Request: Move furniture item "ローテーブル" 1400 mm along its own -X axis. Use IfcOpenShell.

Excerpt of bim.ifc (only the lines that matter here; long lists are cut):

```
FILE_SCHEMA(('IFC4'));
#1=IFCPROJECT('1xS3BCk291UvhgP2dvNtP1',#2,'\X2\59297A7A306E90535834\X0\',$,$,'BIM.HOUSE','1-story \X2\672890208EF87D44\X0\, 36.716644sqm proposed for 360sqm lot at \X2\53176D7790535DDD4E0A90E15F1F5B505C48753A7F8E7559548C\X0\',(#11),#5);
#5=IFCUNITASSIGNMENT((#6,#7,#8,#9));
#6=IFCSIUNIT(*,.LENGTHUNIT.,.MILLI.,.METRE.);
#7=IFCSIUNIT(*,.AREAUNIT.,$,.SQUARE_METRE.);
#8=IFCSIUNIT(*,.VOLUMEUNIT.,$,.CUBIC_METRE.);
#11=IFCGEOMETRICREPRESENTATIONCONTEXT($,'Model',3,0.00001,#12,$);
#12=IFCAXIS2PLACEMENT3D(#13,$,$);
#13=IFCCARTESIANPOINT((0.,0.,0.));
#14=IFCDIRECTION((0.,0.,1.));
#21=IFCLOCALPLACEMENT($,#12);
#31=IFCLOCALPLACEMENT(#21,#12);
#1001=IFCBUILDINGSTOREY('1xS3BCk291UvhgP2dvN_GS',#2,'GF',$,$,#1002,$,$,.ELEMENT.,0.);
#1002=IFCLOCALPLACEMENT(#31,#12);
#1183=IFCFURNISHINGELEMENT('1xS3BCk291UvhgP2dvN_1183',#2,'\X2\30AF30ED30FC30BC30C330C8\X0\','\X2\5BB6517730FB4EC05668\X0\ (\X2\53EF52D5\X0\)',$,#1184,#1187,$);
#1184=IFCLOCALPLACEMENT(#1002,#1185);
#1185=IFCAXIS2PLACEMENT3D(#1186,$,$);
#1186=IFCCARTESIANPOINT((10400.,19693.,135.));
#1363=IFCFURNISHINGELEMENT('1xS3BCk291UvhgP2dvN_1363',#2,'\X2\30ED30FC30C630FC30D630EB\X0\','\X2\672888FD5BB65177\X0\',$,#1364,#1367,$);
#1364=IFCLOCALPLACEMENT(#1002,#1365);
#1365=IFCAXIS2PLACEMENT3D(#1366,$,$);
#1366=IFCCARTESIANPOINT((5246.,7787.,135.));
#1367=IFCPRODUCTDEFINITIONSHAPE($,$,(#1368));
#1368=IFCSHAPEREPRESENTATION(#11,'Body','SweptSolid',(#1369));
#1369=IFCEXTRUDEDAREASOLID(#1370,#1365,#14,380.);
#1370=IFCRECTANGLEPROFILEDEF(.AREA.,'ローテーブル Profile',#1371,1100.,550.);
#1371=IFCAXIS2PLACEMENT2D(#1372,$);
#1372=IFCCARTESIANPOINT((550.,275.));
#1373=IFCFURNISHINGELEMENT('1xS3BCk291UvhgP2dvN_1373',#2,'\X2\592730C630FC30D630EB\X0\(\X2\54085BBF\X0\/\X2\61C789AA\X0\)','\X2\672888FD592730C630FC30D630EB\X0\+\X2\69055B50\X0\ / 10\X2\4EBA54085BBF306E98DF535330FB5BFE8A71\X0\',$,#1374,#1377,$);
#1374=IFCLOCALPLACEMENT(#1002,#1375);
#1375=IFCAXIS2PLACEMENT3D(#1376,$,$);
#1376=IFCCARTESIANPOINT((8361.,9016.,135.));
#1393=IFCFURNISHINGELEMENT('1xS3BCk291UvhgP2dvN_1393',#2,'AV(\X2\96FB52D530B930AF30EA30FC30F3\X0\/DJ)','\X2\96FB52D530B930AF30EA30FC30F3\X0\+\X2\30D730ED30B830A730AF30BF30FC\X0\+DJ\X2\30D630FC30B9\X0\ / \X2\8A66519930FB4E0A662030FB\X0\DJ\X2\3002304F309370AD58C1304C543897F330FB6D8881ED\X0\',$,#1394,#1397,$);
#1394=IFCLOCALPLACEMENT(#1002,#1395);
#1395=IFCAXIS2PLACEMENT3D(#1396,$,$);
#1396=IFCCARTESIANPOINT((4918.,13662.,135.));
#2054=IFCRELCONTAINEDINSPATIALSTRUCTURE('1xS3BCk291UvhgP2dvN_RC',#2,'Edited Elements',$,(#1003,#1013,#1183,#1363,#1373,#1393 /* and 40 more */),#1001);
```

```python
import ifcopenshell
import ifcopenshell.api.geometry
import ifcopenshell.util.placement
import ifcopenshell.util.unit

model = ifcopenshell.open("bim.ifc")
unit_scale = ifcopenshell.util.unit.calculate_unit_scale(model)

item = model.by_id(1363)
matrix = ifcopenshell.util.placement.get_local_placement(item.ObjectPlacement)
matrix[:3, 3] -= matrix[:3, 0] * 1.4 / unit_scale
ifcopenshell.api.geometry.edit_object_placement(model, product=item, matrix=matrix, is_si=False)

print(ifcopenshell.util.placement.get_local_placement(item.ObjectPlacement).round(3) + 0.0)

model.write("bim_updated.ifc")
```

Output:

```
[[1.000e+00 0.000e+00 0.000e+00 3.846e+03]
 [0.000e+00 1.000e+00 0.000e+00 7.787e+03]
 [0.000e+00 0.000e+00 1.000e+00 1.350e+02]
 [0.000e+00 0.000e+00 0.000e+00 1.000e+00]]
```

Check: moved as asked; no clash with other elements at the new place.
